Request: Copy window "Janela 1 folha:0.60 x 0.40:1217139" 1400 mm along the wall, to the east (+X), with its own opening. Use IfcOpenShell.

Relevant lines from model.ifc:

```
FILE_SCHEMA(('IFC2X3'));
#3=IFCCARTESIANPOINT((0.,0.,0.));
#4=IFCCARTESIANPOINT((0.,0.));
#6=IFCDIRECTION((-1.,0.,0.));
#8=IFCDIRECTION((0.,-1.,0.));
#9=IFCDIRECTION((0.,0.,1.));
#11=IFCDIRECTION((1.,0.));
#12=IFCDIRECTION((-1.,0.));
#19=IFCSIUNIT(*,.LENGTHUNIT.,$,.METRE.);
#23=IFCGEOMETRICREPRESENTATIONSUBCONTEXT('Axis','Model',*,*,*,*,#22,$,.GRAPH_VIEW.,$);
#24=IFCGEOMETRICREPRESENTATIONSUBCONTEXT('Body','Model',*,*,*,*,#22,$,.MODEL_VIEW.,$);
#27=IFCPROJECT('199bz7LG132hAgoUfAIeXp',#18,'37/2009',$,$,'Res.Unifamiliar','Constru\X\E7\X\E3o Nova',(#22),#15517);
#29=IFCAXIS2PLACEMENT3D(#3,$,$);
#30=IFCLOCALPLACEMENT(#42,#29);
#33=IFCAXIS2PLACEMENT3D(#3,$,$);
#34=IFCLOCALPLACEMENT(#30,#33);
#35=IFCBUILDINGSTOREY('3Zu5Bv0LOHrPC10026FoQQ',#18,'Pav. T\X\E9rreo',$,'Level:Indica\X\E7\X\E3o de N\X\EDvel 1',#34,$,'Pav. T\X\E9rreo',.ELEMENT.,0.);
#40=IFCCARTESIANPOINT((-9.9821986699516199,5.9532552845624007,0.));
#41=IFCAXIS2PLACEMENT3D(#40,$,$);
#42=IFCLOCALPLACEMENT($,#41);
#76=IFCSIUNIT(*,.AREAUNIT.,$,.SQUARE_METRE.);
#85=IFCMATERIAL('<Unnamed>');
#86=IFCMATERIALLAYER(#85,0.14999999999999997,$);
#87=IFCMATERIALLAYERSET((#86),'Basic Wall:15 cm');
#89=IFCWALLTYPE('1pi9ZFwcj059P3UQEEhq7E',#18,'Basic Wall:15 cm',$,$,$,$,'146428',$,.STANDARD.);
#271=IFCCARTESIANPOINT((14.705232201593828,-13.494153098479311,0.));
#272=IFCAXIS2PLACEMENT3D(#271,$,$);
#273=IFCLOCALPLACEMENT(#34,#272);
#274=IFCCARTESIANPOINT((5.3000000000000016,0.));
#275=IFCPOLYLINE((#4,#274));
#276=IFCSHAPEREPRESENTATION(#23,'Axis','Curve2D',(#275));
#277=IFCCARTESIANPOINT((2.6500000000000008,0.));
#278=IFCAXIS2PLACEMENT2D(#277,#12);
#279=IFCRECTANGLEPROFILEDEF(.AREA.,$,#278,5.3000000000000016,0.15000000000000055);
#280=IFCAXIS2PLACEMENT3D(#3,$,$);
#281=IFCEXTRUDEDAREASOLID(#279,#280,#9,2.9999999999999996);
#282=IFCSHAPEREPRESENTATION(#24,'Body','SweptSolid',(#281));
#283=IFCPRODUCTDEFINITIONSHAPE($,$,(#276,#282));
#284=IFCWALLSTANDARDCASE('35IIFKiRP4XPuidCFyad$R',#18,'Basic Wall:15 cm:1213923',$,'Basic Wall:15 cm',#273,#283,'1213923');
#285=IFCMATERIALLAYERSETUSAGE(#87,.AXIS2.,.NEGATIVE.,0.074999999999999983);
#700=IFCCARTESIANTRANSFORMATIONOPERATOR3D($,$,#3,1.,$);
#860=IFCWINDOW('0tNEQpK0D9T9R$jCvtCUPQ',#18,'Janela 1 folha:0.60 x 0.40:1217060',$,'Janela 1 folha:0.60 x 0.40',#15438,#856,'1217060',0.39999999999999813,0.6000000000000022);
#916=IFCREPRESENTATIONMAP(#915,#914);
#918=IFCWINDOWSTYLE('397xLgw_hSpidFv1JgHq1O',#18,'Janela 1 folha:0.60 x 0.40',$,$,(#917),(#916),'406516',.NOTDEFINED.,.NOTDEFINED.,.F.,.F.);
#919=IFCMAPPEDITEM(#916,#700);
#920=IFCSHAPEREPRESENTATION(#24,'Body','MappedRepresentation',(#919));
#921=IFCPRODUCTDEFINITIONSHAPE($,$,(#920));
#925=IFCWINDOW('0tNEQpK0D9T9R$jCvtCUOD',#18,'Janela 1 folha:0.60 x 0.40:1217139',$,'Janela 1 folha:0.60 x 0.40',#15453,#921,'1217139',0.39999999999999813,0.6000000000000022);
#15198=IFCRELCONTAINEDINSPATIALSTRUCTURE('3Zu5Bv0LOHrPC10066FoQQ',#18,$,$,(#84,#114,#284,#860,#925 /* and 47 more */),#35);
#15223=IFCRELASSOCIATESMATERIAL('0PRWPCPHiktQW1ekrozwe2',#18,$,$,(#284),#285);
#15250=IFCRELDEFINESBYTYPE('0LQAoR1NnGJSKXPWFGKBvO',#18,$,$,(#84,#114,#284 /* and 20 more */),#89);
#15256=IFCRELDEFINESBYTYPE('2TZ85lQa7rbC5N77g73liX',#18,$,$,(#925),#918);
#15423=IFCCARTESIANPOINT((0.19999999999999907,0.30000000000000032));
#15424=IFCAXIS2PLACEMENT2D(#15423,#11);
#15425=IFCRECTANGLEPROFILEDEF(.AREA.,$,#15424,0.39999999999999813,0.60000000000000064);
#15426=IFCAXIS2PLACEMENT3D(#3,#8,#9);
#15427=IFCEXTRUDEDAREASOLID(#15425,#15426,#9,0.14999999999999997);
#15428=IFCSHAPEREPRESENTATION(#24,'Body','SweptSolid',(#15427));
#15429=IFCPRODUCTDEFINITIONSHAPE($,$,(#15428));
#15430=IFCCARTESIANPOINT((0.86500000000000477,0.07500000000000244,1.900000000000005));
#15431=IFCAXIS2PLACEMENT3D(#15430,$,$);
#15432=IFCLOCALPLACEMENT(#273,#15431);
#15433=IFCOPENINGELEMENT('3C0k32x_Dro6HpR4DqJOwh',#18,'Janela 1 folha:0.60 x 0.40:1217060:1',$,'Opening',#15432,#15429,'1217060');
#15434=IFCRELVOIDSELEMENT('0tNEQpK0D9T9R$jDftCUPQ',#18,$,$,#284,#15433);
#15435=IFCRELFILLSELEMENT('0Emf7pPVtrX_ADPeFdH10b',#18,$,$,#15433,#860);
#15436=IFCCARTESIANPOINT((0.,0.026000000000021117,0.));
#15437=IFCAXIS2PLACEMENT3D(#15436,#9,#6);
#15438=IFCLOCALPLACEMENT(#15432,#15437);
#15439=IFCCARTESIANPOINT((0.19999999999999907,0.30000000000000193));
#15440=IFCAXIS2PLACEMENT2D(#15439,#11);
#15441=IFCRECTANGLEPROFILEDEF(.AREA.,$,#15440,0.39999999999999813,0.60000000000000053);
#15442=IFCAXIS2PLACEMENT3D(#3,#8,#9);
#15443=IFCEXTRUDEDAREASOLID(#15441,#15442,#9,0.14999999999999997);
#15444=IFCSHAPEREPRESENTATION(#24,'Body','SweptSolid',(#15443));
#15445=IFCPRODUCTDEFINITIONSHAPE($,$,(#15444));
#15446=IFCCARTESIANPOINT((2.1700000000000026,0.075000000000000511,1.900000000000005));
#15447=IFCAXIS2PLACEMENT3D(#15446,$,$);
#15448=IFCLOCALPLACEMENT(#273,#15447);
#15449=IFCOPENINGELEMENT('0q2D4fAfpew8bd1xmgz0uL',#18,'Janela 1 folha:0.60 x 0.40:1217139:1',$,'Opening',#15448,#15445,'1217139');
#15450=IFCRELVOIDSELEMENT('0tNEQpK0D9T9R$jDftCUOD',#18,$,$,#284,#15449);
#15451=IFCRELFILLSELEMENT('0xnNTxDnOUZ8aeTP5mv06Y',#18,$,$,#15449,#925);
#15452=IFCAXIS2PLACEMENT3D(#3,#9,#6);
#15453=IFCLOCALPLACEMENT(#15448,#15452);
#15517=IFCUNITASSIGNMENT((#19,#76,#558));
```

```python
import ifcopenshell
import ifcopenshell.api.feature
import ifcopenshell.api.geometry
import ifcopenshell.api.root
import ifcopenshell.geom
import ifcopenshell.util.element
import ifcopenshell.util.placement
import ifcopenshell.util.shape
import ifcopenshell.util.unit

model = ifcopenshell.open("model.ifc")
unit_scale = ifcopenshell.util.unit.calculate_unit_scale(model)
settings = ifcopenshell.geom.settings()


def volume(element):
    """Net volume in cubic metres, openings subtracted."""
    shape = ifcopenshell.geom.create_shape(settings, element)
    return ifcopenshell.util.shape.get_volume(shape.geometry)


def reuse_history(source, copy):
    """copy_class also copies each property set's owner history, people and application; keep the originals."""
    for rel in copy.IsDefinedBy:
        if rel.is_a("IfcRelDefinesByProperties") and (history := rel.RelatingPropertyDefinition.OwnerHistory):
            rel.RelatingPropertyDefinition.OwnerHistory = source.OwnerHistory
            ifcopenshell.util.element.remove_deep2(model, history)


window = model.by_guid("0tNEQpK0D9T9R$jCvtCUOD")
opening = window.FillsVoids[0].RelatingOpeningElement
wall = opening.VoidsElements[0].RelatingBuildingElement
before = volume(wall)
shift = ifcopenshell.util.placement.get_local_placement(wall.ObjectPlacement)[:3, 0] * 1.4 / unit_scale

# copy_class copies the void relationship, type, container and properties, but no geometry.
new_opening = ifcopenshell.api.root.copy_class(model, product=opening)
new_opening.Representation = ifcopenshell.util.element.copy_deep(
    model, opening.Representation, exclude=["IfcGeometricRepresentationContext", "IfcRepresentationMap"]
)
new_opening.Name = "Janela 1 folha:0.60 x 0.40"
new_opening.Tag = None
new_window = ifcopenshell.api.root.copy_class(model, product=window)
new_window.Representation = ifcopenshell.util.element.copy_deep(
    model, window.Representation, exclude=["IfcGeometricRepresentationContext", "IfcRepresentationMap"]
)
new_window.Name = "Janela 1 folha:0.60 x 0.40"
new_window.Tag = None
reuse_history(window, new_window)
fills = ifcopenshell.api.feature.add_filling(model, opening=new_opening, element=new_window)
fills.OwnerHistory = new_window.OwnerHistory  # required in IFC2X3

for old, new in ((opening, new_opening), (window, new_window)):
    matrix = ifcopenshell.util.placement.get_local_placement(old.ObjectPlacement)
    matrix[:3, 3] += shift
    ifcopenshell.api.geometry.edit_object_placement(model, product=new, matrix=matrix, is_si=False)

after = volume(wall)

print(f"wall volume {before:.3f} -> {after:.3f} m3")

model.write("model_updated.ifc")
```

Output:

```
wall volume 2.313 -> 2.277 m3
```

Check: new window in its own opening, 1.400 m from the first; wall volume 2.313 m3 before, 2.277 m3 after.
